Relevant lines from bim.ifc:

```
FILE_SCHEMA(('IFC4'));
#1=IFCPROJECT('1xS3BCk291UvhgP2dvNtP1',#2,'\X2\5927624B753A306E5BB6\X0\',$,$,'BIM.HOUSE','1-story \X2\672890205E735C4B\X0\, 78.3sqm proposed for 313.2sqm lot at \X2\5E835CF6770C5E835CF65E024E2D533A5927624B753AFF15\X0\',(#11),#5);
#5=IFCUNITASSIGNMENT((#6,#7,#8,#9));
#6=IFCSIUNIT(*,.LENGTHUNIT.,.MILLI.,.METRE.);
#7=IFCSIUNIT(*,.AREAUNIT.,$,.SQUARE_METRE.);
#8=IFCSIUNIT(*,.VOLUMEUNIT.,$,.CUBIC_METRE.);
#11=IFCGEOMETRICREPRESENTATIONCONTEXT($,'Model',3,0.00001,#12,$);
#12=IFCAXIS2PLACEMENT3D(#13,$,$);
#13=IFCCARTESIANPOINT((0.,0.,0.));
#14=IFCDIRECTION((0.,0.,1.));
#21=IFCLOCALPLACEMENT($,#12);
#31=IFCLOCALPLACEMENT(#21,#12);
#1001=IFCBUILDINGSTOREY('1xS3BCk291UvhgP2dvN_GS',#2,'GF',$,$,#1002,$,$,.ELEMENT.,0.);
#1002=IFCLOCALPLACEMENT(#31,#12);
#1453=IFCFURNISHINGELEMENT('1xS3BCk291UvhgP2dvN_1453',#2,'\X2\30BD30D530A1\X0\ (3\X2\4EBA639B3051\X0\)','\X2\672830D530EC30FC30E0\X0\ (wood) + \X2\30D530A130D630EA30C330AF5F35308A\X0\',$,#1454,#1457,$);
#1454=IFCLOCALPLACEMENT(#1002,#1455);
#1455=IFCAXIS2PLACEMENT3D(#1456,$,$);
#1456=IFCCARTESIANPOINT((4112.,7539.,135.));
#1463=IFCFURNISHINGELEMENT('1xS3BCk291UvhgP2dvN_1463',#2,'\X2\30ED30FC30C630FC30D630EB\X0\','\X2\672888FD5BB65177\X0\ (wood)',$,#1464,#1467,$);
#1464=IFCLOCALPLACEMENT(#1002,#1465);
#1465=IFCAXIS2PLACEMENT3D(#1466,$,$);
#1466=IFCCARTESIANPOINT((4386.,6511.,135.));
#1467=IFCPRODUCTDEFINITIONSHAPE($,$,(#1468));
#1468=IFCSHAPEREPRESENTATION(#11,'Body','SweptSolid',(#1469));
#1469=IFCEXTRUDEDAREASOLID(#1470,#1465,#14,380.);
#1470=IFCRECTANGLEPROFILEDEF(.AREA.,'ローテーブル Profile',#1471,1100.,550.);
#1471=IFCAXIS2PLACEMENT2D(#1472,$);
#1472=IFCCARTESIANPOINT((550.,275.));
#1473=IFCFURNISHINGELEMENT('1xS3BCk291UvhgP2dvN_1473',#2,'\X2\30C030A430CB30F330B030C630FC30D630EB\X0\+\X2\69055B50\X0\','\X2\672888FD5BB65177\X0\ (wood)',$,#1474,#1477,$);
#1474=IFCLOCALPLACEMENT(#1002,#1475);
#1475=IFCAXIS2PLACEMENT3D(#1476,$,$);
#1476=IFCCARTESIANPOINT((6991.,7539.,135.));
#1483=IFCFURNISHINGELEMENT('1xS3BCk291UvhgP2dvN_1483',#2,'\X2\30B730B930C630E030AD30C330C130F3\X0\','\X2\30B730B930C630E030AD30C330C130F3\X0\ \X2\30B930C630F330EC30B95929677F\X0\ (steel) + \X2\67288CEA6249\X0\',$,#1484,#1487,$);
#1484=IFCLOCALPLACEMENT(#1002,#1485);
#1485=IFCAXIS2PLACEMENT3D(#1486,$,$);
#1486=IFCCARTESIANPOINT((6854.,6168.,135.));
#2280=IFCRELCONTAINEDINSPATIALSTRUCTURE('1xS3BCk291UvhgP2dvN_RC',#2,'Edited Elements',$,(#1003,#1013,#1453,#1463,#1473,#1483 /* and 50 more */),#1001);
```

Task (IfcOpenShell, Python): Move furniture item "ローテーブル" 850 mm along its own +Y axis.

```python
import ifcopenshell
import ifcopenshell.api.geometry
import ifcopenshell.util.placement
import ifcopenshell.util.unit

model = ifcopenshell.open("bim.ifc")
unit_scale = ifcopenshell.util.unit.calculate_unit_scale(model)

item = model.by_guid("1xS3BCk291UvhgP2dvN_1463")
matrix = ifcopenshell.util.placement.get_local_placement(item.ObjectPlacement)
matrix[:3, 3] += matrix[:3, 1] * 0.85 / unit_scale
ifcopenshell.api.geometry.edit_object_placement(model, product=item, matrix=matrix, is_si=False)

print(ifcopenshell.util.placement.get_local_placement(item.ObjectPlacement).round(3) + 0.0)

model.write("bim_edited.ifc")
```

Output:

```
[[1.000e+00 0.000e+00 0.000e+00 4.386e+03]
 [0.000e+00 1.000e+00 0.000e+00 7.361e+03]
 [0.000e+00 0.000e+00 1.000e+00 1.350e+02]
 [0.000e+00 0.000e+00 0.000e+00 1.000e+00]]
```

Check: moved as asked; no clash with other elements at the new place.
